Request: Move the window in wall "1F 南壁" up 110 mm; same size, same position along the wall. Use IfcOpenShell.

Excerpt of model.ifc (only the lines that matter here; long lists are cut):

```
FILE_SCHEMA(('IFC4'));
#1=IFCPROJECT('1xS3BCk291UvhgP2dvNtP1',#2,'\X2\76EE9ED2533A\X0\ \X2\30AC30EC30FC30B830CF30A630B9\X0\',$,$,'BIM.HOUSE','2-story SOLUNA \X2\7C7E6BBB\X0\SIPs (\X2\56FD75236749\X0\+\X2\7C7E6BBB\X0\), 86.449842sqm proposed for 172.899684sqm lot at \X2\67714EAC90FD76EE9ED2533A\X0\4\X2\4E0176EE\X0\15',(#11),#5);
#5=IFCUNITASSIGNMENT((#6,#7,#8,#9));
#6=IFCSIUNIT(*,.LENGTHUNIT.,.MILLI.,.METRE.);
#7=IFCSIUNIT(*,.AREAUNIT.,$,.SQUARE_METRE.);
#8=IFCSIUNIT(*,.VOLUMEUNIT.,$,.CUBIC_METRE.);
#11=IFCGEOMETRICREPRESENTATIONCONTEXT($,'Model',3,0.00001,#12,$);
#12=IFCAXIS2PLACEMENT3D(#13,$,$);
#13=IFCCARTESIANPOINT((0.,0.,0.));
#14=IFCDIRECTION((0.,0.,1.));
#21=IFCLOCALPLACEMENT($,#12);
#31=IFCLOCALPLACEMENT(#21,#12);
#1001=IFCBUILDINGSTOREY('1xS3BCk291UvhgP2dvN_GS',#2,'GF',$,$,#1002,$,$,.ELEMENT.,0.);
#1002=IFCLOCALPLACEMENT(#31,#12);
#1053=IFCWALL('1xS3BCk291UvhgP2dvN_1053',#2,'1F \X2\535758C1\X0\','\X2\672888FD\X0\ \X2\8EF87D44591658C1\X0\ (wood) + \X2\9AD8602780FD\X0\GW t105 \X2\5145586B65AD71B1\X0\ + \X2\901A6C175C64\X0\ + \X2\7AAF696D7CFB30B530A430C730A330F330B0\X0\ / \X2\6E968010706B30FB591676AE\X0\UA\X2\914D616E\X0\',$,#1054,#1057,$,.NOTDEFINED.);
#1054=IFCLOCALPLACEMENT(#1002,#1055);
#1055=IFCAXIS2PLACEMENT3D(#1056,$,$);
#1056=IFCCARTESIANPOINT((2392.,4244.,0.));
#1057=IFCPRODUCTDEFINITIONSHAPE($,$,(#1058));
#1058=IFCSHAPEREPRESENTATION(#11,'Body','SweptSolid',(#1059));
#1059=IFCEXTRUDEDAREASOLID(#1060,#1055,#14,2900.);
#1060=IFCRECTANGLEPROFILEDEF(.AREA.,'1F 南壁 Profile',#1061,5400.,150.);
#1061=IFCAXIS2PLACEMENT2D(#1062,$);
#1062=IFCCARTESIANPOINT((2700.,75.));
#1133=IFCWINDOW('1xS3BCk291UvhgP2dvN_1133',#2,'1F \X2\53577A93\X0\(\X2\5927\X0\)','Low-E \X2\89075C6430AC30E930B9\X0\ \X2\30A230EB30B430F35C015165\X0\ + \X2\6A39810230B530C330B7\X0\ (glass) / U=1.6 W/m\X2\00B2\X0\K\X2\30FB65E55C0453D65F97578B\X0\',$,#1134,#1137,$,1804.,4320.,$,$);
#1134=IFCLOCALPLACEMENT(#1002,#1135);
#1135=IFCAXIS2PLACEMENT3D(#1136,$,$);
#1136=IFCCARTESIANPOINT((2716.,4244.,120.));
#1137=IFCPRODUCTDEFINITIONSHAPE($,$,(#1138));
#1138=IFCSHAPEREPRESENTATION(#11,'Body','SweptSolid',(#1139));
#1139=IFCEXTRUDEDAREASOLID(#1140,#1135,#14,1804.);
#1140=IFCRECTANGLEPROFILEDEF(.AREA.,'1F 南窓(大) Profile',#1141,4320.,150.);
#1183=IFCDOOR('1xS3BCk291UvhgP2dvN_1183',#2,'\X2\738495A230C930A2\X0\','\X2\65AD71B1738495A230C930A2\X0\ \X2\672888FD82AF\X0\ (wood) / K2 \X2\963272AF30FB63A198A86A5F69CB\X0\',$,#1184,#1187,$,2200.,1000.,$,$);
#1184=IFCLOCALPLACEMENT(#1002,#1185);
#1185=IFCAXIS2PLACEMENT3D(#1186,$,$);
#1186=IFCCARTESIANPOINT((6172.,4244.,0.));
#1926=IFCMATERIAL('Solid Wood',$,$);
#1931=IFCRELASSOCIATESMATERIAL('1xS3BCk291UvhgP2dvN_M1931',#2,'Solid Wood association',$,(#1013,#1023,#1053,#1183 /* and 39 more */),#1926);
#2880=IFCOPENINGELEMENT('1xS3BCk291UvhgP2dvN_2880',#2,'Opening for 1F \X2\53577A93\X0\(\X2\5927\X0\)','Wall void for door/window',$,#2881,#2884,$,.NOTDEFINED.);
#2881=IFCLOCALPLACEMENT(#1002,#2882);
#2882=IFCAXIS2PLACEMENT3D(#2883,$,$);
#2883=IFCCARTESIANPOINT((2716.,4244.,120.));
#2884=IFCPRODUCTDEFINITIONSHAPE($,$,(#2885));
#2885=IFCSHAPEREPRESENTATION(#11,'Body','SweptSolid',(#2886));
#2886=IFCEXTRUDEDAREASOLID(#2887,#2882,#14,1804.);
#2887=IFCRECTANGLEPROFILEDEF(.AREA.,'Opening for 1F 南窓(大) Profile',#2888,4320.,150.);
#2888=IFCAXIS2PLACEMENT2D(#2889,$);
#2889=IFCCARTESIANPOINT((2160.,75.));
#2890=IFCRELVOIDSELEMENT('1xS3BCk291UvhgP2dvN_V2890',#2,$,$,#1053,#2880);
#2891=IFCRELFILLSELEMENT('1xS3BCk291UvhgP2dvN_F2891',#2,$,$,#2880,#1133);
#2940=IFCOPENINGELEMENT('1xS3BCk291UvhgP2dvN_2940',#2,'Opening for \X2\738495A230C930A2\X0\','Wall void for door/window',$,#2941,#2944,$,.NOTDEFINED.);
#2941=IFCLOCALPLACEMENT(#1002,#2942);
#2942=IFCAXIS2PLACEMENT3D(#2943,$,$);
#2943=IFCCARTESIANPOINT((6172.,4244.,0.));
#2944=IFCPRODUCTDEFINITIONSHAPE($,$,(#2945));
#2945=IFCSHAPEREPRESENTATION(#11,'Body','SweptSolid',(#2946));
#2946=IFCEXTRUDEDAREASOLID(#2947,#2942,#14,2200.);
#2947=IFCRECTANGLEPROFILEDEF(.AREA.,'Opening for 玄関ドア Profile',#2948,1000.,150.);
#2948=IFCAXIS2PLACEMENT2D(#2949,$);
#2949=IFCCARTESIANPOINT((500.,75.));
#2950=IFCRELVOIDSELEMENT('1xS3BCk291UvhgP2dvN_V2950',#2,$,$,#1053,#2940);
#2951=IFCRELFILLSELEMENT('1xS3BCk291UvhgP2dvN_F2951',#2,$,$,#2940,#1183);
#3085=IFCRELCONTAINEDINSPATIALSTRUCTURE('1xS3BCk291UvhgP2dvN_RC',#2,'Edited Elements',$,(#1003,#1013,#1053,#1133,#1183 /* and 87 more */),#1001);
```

```python
import numpy as np
import ifcopenshell
import ifcopenshell.api.geometry
import ifcopenshell.util.placement
import ifcopenshell.util.unit

model = ifcopenshell.open("model.ifc")
unit_scale = ifcopenshell.util.unit.calculate_unit_scale(model)

window = model.by_guid("1xS3BCk291UvhgP2dvN_1133")
opening = window.FillsVoids[0].RelatingOpeningElement
dz = 0.11 / unit_scale

shift = np.array([0.0, 0.0, dz])
# The window is not placed relative to its opening, so move both.
for product in (opening, window):
    matrix = ifcopenshell.util.placement.get_local_placement(product.ObjectPlacement)
    matrix[:3, 3] += shift
    ifcopenshell.api.geometry.edit_object_placement(model, product=product, matrix=matrix, is_si=False)

print(f"moved by {dz * unit_scale:+.3f} m")

model.write("model_edited.ifc")
```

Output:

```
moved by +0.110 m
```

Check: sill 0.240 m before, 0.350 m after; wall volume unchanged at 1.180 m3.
